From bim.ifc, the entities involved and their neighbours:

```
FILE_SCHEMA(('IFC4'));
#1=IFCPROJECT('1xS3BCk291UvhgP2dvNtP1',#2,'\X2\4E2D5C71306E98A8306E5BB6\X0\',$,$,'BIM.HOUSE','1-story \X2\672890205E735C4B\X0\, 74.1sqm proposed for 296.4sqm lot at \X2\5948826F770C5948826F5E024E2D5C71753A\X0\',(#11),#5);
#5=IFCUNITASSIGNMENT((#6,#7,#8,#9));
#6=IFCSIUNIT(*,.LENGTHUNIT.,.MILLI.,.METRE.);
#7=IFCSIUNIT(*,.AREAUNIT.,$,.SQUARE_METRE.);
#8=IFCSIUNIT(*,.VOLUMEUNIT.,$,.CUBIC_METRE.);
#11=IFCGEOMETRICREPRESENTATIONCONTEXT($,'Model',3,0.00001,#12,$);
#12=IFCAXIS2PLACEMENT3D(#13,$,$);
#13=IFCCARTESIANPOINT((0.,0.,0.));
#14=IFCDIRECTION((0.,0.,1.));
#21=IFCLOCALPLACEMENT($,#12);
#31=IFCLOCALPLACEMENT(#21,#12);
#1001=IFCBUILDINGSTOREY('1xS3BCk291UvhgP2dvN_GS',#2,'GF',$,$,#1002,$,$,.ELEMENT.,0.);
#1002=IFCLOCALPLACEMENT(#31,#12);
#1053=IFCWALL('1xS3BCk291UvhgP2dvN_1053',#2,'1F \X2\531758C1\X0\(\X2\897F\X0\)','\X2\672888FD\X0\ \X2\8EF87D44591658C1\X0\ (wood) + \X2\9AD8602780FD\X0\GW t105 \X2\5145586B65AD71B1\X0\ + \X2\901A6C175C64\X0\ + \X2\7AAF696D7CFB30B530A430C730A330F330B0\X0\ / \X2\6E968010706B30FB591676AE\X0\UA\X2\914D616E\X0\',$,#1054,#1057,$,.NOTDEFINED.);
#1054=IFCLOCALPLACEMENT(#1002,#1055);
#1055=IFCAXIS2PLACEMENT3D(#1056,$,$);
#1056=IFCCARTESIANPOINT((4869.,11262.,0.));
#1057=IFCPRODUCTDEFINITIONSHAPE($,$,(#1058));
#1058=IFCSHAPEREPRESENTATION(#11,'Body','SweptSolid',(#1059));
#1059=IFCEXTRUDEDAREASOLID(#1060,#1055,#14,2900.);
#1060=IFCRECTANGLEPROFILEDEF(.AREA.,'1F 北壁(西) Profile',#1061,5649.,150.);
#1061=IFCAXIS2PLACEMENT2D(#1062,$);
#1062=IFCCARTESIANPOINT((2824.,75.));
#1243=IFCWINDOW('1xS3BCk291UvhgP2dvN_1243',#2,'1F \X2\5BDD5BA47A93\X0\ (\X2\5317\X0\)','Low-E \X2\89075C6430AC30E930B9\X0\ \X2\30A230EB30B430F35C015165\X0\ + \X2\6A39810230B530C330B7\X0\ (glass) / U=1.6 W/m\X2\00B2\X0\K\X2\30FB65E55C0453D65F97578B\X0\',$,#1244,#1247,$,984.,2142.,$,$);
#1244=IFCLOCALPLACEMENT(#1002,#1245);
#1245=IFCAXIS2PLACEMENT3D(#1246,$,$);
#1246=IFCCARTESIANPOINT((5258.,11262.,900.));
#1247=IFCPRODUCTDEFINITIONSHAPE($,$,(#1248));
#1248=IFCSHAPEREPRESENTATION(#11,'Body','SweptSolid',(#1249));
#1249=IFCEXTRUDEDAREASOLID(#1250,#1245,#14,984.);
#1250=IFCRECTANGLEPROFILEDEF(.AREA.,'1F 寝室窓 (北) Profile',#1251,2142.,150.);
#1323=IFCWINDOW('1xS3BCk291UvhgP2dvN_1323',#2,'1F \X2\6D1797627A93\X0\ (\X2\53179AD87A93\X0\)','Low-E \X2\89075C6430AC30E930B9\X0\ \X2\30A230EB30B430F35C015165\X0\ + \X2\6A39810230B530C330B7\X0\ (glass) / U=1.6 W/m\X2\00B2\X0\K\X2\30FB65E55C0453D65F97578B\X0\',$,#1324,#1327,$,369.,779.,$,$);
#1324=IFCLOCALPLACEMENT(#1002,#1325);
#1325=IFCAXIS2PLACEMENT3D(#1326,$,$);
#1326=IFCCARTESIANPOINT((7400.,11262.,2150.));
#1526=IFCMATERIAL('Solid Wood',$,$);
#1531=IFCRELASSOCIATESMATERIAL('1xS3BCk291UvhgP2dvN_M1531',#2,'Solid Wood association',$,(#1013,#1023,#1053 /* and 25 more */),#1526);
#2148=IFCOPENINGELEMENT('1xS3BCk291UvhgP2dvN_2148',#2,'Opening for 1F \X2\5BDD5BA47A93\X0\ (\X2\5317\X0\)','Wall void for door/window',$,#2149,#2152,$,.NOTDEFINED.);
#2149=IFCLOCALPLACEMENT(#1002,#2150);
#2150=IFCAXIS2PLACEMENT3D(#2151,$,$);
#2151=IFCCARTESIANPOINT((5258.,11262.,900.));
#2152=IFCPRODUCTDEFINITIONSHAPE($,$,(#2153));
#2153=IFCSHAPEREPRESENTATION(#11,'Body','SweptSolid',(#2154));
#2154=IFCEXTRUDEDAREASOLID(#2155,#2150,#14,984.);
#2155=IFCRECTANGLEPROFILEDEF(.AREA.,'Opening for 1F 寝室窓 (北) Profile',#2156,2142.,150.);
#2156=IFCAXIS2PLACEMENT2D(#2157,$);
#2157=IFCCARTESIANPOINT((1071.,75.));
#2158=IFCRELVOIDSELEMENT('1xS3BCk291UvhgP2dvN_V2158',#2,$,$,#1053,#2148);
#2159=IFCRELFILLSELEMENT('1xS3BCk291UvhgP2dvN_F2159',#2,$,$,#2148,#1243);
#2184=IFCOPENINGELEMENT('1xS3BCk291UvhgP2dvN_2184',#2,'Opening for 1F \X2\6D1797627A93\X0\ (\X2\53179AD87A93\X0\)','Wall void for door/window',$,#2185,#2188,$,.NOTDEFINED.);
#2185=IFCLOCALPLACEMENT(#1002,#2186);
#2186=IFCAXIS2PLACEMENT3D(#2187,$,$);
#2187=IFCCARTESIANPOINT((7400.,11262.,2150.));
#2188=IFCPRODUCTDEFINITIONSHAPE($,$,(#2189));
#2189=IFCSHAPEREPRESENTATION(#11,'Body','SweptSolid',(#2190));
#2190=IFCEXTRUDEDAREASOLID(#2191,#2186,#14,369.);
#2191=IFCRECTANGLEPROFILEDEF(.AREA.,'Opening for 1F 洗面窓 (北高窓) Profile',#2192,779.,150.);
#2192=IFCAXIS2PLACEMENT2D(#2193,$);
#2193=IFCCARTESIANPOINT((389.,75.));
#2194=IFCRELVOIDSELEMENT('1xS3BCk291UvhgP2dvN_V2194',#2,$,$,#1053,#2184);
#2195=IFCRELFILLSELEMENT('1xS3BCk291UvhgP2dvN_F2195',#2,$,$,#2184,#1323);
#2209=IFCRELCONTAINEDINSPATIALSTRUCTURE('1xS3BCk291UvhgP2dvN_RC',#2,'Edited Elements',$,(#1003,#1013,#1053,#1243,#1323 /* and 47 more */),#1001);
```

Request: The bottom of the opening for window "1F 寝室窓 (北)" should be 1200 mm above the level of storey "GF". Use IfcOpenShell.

```python
import numpy as np
import ifcopenshell
import ifcopenshell.api.geometry
import ifcopenshell.geom
import ifcopenshell.util.element
import ifcopenshell.util.placement
import ifcopenshell.util.shape
import ifcopenshell.util.unit

model = ifcopenshell.open("bim.ifc")
unit_scale = ifcopenshell.util.unit.calculate_unit_scale(model)

window = model.by_guid("1xS3BCk291UvhgP2dvN_1243")
opening = window.FillsVoids[0].RelatingOpeningElement
storey = ifcopenshell.util.element.get_container(window, ifc_class="IfcBuildingStorey")
level = ifcopenshell.util.placement.get_local_placement(storey.ObjectPlacement)[2, 3]

# The opening's origin need not be at the sill, so measure its lowest point.
shape = ifcopenshell.geom.create_shape(ifcopenshell.geom.settings(), opening)
bottom = ifcopenshell.util.shape.get_shape_bottom_elevation(shape, shape.geometry) / unit_scale
dz = level + 1200.0 - bottom

shift = np.array([0.0, 0.0, dz])
# The window is not placed relative to its opening, so move both.
for product in (opening, window):
    matrix = ifcopenshell.util.placement.get_local_placement(product.ObjectPlacement)
    matrix[:3, 3] += shift
    ifcopenshell.api.geometry.edit_object_placement(model, product=product, matrix=matrix, is_si=False)

print(f"moved by {dz * unit_scale:+.3f} m")

model.write("bim_rev.ifc")
```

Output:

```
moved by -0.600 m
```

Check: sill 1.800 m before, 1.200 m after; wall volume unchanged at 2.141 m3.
